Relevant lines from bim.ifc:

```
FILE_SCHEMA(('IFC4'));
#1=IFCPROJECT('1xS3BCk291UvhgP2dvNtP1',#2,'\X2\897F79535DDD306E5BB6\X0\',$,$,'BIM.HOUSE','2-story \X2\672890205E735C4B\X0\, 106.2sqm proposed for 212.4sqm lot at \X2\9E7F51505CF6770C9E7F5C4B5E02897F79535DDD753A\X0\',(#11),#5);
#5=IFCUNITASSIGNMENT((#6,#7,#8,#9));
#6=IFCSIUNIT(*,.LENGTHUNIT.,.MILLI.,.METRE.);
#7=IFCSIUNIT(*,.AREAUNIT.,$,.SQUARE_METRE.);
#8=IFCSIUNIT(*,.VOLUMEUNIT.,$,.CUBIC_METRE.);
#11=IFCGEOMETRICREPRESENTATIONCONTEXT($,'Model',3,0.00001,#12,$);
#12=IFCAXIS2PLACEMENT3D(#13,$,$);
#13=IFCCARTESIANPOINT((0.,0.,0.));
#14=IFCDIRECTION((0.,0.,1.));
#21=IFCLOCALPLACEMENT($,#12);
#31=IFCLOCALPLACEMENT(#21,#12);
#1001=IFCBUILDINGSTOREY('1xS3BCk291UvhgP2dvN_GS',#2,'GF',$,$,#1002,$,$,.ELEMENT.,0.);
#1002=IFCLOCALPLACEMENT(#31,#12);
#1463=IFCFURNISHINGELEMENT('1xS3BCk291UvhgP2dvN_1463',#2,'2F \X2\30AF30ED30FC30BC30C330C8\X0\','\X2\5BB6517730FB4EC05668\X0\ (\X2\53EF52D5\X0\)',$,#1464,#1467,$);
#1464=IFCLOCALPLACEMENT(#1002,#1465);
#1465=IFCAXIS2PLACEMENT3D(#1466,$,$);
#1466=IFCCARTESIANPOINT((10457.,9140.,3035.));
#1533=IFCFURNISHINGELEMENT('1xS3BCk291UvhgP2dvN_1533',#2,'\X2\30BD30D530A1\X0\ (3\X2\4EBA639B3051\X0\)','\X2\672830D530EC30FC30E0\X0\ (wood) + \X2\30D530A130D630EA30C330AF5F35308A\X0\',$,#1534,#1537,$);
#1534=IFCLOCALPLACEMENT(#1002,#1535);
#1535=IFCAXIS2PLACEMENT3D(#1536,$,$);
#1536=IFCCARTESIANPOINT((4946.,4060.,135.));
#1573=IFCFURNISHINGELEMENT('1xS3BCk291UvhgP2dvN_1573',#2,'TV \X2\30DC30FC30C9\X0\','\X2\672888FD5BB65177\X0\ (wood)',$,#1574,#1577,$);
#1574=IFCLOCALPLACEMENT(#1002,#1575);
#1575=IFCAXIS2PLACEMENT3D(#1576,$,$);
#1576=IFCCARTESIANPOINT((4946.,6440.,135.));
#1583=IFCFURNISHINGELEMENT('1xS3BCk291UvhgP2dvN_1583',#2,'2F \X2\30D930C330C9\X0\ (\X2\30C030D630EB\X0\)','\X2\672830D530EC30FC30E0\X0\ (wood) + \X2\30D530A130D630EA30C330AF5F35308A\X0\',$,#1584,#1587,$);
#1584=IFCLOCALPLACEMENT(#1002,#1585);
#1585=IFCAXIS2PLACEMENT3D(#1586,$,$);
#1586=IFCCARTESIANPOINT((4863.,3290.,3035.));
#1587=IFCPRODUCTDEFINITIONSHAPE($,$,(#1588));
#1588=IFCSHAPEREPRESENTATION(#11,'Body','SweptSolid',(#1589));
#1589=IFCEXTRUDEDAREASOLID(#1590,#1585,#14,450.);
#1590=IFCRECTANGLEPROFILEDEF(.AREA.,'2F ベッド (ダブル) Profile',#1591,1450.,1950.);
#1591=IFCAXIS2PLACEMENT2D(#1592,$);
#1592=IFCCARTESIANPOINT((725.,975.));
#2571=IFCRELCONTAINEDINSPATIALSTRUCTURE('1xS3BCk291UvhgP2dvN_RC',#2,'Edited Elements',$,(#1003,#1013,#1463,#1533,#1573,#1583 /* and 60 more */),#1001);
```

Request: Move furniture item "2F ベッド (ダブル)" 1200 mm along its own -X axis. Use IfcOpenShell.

```python
import ifcopenshell
import ifcopenshell.api.geometry
import ifcopenshell.util.placement
import ifcopenshell.util.unit

model = ifcopenshell.open("bim.ifc")
unit_scale = ifcopenshell.util.unit.calculate_unit_scale(model)

item = model.by_id(1583)
matrix = ifcopenshell.util.placement.get_local_placement(item.ObjectPlacement)
matrix[:3, 3] -= matrix[:3, 0] * 1.2 / unit_scale
ifcopenshell.api.geometry.edit_object_placement(model, product=item, matrix=matrix, is_si=False)

print(ifcopenshell.util.placement.get_local_placement(item.ObjectPlacement).round(3) + 0.0)

model.write("bim_edited.ifc")
```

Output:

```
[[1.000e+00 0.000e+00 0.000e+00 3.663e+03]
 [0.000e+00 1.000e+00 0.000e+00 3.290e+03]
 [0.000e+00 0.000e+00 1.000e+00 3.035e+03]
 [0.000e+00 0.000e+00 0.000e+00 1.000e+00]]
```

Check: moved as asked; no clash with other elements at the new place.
